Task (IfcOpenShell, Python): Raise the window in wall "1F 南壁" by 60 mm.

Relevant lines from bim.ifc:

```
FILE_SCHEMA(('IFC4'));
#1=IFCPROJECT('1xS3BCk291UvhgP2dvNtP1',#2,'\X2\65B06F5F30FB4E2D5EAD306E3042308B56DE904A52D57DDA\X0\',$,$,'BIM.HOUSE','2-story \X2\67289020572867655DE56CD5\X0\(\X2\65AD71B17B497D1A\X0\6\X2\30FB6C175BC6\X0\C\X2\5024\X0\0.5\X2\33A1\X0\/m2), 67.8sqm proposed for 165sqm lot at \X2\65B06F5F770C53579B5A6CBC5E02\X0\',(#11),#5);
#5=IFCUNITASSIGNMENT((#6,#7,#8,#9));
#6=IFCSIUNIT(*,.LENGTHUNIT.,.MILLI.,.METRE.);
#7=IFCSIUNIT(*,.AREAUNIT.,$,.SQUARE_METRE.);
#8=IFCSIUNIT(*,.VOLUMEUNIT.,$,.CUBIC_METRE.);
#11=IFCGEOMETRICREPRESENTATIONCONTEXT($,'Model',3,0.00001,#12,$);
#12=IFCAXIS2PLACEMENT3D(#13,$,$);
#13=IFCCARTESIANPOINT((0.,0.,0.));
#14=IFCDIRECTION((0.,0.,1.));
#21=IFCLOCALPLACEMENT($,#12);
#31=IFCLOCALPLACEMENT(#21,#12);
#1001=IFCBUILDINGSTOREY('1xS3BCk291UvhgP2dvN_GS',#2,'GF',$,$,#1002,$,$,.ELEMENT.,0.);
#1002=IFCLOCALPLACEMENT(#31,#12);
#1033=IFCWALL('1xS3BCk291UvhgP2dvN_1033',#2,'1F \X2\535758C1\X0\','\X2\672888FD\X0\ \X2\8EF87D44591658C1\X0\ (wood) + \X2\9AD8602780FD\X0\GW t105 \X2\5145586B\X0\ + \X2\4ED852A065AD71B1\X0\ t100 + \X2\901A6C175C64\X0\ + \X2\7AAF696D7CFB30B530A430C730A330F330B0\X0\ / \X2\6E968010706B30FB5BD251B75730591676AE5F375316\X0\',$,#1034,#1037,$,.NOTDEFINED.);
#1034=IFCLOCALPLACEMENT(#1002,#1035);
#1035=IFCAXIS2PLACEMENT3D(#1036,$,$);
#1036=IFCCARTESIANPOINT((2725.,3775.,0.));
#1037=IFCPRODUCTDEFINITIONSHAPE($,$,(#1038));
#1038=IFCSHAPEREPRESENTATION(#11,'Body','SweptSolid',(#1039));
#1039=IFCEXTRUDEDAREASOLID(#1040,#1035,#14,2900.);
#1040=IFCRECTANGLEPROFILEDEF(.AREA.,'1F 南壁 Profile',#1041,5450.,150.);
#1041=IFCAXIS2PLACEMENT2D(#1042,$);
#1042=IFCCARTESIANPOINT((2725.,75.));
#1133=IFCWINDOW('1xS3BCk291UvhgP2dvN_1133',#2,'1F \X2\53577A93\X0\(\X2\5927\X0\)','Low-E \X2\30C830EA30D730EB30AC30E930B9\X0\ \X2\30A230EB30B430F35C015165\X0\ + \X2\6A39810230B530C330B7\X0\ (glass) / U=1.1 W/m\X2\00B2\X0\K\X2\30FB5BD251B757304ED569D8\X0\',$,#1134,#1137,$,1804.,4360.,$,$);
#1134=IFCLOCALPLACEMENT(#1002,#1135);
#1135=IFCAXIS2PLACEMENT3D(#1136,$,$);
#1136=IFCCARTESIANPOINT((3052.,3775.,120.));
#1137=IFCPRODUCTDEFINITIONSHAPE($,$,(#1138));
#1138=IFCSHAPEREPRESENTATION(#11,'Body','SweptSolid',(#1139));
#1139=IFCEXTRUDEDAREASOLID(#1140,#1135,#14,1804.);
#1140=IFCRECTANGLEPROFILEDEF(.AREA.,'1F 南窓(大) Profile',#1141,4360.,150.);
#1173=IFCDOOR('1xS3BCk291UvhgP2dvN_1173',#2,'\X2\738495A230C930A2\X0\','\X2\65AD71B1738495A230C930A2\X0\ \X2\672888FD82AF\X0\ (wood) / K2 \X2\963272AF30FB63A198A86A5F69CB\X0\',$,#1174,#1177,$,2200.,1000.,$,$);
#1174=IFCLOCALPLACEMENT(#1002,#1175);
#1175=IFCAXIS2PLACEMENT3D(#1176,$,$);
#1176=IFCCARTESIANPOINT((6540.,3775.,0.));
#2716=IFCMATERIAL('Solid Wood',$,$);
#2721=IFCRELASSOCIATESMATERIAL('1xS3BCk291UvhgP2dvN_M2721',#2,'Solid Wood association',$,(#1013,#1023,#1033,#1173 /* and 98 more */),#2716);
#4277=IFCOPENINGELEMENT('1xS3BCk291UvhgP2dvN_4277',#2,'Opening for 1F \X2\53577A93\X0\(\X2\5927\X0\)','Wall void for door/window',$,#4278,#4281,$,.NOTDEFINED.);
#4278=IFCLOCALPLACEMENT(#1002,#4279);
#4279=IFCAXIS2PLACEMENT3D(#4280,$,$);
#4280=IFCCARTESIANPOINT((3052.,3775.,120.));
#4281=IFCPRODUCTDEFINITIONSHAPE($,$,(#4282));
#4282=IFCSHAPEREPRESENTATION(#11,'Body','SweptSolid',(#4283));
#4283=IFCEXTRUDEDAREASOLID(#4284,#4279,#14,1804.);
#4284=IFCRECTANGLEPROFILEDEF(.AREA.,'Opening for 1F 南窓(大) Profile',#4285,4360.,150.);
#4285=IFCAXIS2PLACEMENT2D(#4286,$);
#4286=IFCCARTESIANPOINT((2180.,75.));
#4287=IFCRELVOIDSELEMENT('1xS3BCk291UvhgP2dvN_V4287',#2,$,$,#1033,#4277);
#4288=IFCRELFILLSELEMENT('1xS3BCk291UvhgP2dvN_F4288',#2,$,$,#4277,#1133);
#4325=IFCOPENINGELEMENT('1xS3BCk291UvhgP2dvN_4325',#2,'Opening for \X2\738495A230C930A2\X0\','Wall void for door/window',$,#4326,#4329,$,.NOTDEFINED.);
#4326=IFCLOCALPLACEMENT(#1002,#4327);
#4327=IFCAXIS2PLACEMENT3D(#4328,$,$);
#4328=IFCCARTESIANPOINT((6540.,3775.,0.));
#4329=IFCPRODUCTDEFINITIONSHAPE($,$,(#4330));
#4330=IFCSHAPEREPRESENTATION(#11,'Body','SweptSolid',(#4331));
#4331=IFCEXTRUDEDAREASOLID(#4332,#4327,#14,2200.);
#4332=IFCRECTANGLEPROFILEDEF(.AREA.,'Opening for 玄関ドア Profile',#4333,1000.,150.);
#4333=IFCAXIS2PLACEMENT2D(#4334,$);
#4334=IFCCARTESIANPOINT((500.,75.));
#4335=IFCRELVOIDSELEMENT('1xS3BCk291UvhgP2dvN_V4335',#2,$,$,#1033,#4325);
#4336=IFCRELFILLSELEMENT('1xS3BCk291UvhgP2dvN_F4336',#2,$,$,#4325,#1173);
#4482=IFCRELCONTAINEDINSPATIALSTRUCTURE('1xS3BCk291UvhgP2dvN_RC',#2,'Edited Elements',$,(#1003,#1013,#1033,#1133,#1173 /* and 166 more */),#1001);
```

```python
import numpy as np
import ifcopenshell
import ifcopenshell.api.geometry
import ifcopenshell.util.placement
import ifcopenshell.util.unit

model = ifcopenshell.open("bim.ifc")
unit_scale = ifcopenshell.util.unit.calculate_unit_scale(model)

window = model.by_guid("1xS3BCk291UvhgP2dvN_1133")
opening = window.FillsVoids[0].RelatingOpeningElement
dz = 60.0

shift = np.array([0.0, 0.0, dz])
# The window is not placed relative to its opening, so move both.
for product in (opening, window):
    matrix = ifcopenshell.util.placement.get_local_placement(product.ObjectPlacement)
    matrix[:3, 3] += shift
    ifcopenshell.api.geometry.edit_object_placement(model, product=product, matrix=matrix, is_si=False)

print(f"moved by {dz * unit_scale:+.3f} m")

model.write("bim-out.ifc")
```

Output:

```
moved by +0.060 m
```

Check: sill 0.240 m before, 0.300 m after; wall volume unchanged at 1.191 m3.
